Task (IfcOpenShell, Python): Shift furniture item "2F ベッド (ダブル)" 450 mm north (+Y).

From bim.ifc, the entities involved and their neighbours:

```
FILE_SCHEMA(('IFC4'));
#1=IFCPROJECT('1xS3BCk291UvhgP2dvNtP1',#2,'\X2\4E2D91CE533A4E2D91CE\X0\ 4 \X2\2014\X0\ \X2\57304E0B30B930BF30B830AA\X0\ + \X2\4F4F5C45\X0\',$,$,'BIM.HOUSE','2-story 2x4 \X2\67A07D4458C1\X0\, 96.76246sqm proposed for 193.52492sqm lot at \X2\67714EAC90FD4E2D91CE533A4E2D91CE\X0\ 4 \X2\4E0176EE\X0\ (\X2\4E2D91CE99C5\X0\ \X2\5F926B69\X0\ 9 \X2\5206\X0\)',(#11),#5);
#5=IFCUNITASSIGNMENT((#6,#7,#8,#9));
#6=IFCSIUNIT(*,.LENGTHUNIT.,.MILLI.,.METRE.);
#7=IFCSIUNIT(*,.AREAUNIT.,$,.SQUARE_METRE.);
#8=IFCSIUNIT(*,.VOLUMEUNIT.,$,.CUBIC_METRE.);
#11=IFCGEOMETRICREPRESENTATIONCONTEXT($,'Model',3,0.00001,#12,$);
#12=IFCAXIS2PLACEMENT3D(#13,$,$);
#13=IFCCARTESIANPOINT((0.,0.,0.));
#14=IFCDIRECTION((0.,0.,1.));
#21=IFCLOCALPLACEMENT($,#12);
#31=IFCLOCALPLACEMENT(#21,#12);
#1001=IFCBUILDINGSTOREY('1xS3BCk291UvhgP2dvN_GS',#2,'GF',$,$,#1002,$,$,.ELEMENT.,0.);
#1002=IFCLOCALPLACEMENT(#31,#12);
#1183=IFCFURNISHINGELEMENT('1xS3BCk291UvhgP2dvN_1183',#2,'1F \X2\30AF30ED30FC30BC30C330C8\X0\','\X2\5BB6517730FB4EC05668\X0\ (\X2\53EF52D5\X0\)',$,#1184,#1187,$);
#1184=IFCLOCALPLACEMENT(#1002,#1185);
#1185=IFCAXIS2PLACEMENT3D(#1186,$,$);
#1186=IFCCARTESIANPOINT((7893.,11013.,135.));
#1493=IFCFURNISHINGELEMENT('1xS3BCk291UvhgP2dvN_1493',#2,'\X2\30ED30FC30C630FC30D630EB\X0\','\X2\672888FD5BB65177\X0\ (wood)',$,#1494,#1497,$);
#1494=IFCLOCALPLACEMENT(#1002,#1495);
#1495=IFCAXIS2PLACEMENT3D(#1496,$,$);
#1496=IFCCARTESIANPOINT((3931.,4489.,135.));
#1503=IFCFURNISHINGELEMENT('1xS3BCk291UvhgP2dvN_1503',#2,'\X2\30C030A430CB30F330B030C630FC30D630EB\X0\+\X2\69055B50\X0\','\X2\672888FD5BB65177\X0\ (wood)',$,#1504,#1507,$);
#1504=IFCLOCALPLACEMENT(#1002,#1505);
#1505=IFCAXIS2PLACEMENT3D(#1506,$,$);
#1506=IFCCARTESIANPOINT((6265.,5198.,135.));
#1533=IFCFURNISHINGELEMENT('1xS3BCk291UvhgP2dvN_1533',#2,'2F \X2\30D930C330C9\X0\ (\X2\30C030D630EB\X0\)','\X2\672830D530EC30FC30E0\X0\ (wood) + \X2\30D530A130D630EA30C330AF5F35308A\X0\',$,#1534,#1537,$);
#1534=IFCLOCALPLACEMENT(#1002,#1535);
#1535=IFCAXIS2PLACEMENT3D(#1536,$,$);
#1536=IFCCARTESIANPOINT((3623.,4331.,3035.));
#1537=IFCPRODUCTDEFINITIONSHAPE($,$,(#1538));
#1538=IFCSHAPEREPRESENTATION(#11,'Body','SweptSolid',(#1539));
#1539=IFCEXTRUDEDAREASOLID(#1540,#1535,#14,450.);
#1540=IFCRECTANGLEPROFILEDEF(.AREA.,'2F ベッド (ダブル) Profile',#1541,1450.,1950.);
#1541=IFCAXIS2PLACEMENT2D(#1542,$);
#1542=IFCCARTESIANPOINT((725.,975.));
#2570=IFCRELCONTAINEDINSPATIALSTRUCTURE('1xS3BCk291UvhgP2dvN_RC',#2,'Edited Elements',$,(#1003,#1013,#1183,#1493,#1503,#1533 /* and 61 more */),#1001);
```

```python
import ifcopenshell
import ifcopenshell.api.geometry
import ifcopenshell.util.placement
import ifcopenshell.util.unit

model = ifcopenshell.open("bim.ifc")
unit_scale = ifcopenshell.util.unit.calculate_unit_scale(model)

item = model.by_id(1533)
matrix = ifcopenshell.util.placement.get_local_placement(item.ObjectPlacement)
matrix[1, 3] += 0.45 / unit_scale
ifcopenshell.api.geometry.edit_object_placement(model, product=item, matrix=matrix, is_si=False)

print(ifcopenshell.util.placement.get_local_placement(item.ObjectPlacement).round(3) + 0.0)

model.write("bim_rev.ifc")
```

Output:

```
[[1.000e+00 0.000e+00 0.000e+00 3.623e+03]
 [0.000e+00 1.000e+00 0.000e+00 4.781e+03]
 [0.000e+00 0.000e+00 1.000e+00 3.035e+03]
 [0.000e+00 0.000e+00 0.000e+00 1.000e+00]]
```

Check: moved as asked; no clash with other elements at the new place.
